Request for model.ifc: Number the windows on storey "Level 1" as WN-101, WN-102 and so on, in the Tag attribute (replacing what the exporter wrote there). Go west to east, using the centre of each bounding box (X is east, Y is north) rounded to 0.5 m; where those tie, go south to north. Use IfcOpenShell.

First a look at what the model holds.

```python
import ifcopenshell
import ifcopenshell.util.element
import ifcopenshell.util.placement

model = ifcopenshell.open("model.ifc")
print(model.schema)
storey = next(s for s in model.by_type("IfcBuildingStorey") if s.Name == "Level 1")
windows = [e for e in ifcopenshell.util.element.get_decomposition(storey) if e.is_a("IfcWindow")]
for e in sorted(windows, key=lambda e: e.id()):
    origin = ifcopenshell.util.placement.get_local_placement(e.ObjectPlacement)[:3, 3]
    print(e.id(), e.Tag, e.Name, origin.round(2) + 0.0, sep=" | ")
```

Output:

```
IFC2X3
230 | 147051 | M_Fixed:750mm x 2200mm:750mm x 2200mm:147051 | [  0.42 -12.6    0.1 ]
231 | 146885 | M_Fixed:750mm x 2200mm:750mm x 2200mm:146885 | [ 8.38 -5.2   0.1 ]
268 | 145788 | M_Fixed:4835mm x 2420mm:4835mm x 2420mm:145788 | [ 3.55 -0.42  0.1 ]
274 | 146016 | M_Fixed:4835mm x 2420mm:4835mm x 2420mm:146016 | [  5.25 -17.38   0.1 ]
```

```python
import ifcopenshell
import ifcopenshell.geom
import ifcopenshell.util.element
import ifcopenshell.util.shape

model = ifcopenshell.open("model.ifc")
settings = ifcopenshell.geom.settings()
settings.set("use-world-coords", True)


def centre(element):
    shape = ifcopenshell.geom.create_shape(settings, element)
    return ifcopenshell.util.shape.get_bbox_centroid(shape.geometry)


storey = next(s for s in model.by_type("IfcBuildingStorey") if s.Name == "Level 1")
windows = [e for e in ifcopenshell.util.element.get_decomposition(storey) if e.is_a("IfcWindow")]

# Insertion points can sit at a corner or the storey origin, so sort by the geometry (in metres).
centres = {e: centre(e) for e in windows}
windows.sort(key=lambda e: (round(centres[e][0] / 0.5), centres[e][1]))

for i, e in enumerate(windows, start=1):
    number = f"WN-1{i:02d}"
    e.Tag = number
    print(e.id(), number)

model.write("model-out.ifc")
```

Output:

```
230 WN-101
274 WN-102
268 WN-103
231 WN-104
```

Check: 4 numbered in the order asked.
